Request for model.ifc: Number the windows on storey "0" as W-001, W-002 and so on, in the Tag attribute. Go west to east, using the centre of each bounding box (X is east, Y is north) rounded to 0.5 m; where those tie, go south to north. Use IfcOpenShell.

First a look at what the model holds.

```python
import ifcopenshell
import ifcopenshell.util.element
import ifcopenshell.util.placement

model = ifcopenshell.open("model.ifc")
print(model.schema)
storey = next(s for s in model.by_type("IfcBuildingStorey") if s.Name == "0")
windows = [e for e in ifcopenshell.util.element.get_decomposition(storey) if e.is_a("IfcWindow")]
for e in sorted(windows, key=lambda e: e.id()):
    origin = ifcopenshell.util.placement.get_local_placement(e.ObjectPlacement)[:3, 3]
    print(e.id(), e.Tag, e.Name, origin.round(2) + 0.0, sep=" | ")
```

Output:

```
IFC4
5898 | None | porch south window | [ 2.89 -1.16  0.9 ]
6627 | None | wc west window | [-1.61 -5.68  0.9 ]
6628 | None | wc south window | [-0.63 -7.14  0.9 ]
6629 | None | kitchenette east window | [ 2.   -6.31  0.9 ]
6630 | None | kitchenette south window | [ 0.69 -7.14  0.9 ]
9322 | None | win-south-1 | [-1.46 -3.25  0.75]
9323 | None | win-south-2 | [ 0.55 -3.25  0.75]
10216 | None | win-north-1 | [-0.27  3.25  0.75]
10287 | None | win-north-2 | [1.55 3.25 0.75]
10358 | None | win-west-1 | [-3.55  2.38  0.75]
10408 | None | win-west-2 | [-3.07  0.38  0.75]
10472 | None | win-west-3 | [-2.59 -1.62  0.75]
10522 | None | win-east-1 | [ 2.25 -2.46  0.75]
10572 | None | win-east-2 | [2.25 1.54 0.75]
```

```python
import ifcopenshell
import ifcopenshell.geom
import ifcopenshell.util.element
import ifcopenshell.util.shape

model = ifcopenshell.open("model.ifc")
settings = ifcopenshell.geom.settings()
settings.set("use-world-coords", True)


def centre(element):
    shape = ifcopenshell.geom.create_shape(settings, element)
    return ifcopenshell.util.shape.get_bbox_centroid(shape.geometry)


storey = next(s for s in model.by_type("IfcBuildingStorey") if s.Name == "0")
windows = [e for e in ifcopenshell.util.element.get_decomposition(storey) if e.is_a("IfcWindow")]

# Insertion points can sit at a corner or the storey origin, so sort by the geometry (in metres).
centres = {e: centre(e) for e in windows}
windows.sort(key=lambda e: (round(centres[e][0] / 0.5), centres[e][1]))

for i, e in enumerate(windows, start=1):
    number = f"W-0{i:02d}"
    e.Tag = number
    print(e.id(), number)

model.write("model_updated.ifc")
```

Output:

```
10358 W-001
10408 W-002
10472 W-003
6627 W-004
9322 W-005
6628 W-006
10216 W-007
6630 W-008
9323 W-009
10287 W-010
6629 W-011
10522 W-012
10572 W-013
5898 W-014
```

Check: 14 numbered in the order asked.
